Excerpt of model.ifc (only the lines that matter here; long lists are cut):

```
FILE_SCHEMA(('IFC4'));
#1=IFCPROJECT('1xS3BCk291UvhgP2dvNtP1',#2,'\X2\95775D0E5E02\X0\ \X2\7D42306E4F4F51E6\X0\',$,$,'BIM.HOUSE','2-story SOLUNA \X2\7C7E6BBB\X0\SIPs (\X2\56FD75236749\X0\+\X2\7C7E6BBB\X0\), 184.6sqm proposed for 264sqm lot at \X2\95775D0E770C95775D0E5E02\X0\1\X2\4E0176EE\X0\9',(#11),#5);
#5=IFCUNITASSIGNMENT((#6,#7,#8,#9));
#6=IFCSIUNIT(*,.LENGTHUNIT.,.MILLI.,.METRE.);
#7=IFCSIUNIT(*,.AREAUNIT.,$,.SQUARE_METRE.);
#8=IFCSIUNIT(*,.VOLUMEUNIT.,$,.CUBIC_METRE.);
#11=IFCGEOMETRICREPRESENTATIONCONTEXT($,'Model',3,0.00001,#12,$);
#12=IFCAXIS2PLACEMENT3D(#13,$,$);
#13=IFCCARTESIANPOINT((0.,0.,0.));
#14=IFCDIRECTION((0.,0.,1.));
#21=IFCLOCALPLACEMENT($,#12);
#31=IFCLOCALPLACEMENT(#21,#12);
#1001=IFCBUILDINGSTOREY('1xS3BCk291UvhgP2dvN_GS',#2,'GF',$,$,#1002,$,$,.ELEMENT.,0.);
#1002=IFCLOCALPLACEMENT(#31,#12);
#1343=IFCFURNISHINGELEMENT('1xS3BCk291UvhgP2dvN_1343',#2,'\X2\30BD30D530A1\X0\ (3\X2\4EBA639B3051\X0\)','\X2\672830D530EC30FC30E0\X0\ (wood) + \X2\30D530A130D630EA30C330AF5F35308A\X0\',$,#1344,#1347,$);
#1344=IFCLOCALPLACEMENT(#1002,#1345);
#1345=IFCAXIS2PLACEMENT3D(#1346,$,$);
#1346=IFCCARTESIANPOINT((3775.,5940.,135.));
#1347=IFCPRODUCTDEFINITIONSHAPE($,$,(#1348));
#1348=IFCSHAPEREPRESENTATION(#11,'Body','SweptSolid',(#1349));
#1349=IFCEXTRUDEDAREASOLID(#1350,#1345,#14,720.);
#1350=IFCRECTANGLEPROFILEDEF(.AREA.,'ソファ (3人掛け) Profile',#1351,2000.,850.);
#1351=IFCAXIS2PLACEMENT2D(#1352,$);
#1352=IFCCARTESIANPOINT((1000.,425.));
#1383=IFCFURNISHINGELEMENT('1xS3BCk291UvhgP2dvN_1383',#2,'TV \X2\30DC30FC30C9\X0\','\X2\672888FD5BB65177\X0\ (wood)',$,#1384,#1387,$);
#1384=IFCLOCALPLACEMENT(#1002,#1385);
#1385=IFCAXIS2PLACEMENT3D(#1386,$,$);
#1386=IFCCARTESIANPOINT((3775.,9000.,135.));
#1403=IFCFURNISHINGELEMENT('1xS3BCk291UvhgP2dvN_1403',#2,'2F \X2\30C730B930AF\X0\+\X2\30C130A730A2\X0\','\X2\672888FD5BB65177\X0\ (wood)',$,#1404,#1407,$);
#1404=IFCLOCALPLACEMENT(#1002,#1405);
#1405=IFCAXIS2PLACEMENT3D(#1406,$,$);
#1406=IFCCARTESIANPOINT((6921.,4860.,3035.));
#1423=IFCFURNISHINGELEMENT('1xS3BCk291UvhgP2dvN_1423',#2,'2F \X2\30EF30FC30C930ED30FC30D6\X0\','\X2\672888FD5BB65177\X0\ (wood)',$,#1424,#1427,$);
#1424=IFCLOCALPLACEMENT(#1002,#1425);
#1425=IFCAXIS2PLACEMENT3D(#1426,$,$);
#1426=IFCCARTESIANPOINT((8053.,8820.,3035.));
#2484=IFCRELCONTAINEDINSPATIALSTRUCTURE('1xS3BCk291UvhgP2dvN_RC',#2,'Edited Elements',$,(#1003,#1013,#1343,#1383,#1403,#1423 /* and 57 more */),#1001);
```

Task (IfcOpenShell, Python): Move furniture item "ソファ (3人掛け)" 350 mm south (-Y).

```python
import ifcopenshell
import ifcopenshell.api.geometry
import ifcopenshell.util.placement

model = ifcopenshell.open("model.ifc")

item = model.by_guid("1xS3BCk291UvhgP2dvN_1343")
matrix = ifcopenshell.util.placement.get_local_placement(item.ObjectPlacement)
matrix[1, 3] -= 350.0
ifcopenshell.api.geometry.edit_object_placement(model, product=item, matrix=matrix, is_si=False)

print(ifcopenshell.util.placement.get_local_placement(item.ObjectPlacement).round(3) + 0.0)

model.write("model_updated.ifc")
```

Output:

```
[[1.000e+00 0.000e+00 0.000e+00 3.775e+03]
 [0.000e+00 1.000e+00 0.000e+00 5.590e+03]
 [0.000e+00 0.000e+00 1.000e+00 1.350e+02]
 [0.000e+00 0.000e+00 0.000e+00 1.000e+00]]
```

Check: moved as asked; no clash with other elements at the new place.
